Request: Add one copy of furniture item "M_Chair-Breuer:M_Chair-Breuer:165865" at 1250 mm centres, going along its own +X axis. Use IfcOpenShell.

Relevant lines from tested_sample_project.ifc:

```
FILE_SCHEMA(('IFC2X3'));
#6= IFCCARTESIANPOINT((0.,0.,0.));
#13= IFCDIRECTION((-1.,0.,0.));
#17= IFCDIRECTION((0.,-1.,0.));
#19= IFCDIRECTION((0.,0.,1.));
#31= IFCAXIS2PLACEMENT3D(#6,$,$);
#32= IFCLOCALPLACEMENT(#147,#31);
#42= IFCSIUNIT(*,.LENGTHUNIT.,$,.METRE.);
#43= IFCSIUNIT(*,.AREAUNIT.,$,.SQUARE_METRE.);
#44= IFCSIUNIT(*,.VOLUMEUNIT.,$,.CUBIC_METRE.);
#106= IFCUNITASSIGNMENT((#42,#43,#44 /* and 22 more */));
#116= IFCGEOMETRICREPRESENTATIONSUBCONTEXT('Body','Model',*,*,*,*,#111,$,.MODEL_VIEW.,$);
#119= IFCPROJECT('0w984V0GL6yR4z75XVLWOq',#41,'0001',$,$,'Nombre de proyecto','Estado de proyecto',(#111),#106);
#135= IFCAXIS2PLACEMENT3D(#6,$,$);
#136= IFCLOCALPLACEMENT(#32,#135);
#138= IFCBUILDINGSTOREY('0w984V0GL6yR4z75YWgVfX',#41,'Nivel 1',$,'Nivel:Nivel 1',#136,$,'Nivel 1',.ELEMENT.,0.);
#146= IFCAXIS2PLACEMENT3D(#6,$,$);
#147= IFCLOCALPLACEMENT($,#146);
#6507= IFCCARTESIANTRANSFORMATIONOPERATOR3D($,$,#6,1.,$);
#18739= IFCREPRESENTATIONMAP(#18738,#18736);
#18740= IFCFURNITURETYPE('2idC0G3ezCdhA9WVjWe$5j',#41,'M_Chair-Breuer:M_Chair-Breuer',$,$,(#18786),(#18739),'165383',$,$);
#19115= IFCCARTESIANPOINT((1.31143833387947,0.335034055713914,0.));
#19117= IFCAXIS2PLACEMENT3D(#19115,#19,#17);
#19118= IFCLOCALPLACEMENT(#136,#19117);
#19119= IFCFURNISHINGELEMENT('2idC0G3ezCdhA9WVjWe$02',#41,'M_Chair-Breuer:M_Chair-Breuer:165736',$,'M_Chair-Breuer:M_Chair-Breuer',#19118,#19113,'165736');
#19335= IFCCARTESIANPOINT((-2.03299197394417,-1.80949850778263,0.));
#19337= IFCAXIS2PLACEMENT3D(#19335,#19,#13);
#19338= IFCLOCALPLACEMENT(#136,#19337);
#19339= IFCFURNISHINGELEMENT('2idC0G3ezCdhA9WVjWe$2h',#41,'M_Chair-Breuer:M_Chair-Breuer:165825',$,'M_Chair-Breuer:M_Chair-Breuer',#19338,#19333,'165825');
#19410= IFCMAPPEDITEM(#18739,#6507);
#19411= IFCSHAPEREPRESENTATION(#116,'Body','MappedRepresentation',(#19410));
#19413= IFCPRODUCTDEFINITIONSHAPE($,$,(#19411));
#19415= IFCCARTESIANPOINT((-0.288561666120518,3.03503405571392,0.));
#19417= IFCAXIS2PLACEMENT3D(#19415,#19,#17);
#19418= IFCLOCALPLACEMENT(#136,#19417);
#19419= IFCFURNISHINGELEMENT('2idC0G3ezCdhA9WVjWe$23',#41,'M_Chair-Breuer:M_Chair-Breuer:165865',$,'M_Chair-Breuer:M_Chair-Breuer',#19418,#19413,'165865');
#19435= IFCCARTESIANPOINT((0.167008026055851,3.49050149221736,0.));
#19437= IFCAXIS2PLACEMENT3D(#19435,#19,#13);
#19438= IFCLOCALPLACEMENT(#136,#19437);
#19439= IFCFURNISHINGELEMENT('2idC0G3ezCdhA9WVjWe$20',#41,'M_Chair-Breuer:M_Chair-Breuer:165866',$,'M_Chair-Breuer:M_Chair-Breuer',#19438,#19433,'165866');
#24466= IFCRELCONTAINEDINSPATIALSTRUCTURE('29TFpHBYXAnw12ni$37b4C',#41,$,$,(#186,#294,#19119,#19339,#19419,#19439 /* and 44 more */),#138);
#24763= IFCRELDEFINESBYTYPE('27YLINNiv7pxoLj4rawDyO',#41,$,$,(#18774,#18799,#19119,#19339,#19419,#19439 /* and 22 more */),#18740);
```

```python
import ifcopenshell
import ifcopenshell.api.geometry
import ifcopenshell.api.root
import ifcopenshell.util.element
import ifcopenshell.util.placement
import ifcopenshell.util.unit

model = ifcopenshell.open("tested_sample_project.ifc")
unit_scale = ifcopenshell.util.unit.calculate_unit_scale(model)


def reuse_history(source, copy):
    """copy_class also copies each property set's owner history, people and application; keep the originals."""
    for rel in copy.IsDefinedBy:
        if rel.is_a("IfcRelDefinesByProperties") and (history := rel.RelatingPropertyDefinition.OwnerHistory):
            rel.RelatingPropertyDefinition.OwnerHistory = source.OwnerHistory
            ifcopenshell.util.element.remove_deep2(model, history)


source = model.by_guid("2idC0G3ezCdhA9WVjWe$23")
base = ifcopenshell.util.placement.get_local_placement(source.ObjectPlacement)
step = base[:3, 0] * 1.25 / unit_scale

for i in range(1, 2):
    copy = ifcopenshell.api.root.copy_class(model, product=source)
    copy.Representation = ifcopenshell.util.element.copy_deep(
        model, source.Representation, exclude=["IfcGeometricRepresentationContext", "IfcRepresentationMap"]
    )
    copy.Name = "M_Chair-Breuer:M_Chair-Breuer"
    copy.Tag = None
    reuse_history(source, copy)
    matrix = base.copy()
    matrix[:3, 3] += i * step
    print("added at", matrix[:3, 3].round(3) + 0.0)
    ifcopenshell.api.geometry.edit_object_placement(model, product=copy, matrix=matrix, is_si=False)

model.write("tested_sample_project_rev.ifc")
```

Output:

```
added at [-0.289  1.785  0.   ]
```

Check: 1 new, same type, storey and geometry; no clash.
